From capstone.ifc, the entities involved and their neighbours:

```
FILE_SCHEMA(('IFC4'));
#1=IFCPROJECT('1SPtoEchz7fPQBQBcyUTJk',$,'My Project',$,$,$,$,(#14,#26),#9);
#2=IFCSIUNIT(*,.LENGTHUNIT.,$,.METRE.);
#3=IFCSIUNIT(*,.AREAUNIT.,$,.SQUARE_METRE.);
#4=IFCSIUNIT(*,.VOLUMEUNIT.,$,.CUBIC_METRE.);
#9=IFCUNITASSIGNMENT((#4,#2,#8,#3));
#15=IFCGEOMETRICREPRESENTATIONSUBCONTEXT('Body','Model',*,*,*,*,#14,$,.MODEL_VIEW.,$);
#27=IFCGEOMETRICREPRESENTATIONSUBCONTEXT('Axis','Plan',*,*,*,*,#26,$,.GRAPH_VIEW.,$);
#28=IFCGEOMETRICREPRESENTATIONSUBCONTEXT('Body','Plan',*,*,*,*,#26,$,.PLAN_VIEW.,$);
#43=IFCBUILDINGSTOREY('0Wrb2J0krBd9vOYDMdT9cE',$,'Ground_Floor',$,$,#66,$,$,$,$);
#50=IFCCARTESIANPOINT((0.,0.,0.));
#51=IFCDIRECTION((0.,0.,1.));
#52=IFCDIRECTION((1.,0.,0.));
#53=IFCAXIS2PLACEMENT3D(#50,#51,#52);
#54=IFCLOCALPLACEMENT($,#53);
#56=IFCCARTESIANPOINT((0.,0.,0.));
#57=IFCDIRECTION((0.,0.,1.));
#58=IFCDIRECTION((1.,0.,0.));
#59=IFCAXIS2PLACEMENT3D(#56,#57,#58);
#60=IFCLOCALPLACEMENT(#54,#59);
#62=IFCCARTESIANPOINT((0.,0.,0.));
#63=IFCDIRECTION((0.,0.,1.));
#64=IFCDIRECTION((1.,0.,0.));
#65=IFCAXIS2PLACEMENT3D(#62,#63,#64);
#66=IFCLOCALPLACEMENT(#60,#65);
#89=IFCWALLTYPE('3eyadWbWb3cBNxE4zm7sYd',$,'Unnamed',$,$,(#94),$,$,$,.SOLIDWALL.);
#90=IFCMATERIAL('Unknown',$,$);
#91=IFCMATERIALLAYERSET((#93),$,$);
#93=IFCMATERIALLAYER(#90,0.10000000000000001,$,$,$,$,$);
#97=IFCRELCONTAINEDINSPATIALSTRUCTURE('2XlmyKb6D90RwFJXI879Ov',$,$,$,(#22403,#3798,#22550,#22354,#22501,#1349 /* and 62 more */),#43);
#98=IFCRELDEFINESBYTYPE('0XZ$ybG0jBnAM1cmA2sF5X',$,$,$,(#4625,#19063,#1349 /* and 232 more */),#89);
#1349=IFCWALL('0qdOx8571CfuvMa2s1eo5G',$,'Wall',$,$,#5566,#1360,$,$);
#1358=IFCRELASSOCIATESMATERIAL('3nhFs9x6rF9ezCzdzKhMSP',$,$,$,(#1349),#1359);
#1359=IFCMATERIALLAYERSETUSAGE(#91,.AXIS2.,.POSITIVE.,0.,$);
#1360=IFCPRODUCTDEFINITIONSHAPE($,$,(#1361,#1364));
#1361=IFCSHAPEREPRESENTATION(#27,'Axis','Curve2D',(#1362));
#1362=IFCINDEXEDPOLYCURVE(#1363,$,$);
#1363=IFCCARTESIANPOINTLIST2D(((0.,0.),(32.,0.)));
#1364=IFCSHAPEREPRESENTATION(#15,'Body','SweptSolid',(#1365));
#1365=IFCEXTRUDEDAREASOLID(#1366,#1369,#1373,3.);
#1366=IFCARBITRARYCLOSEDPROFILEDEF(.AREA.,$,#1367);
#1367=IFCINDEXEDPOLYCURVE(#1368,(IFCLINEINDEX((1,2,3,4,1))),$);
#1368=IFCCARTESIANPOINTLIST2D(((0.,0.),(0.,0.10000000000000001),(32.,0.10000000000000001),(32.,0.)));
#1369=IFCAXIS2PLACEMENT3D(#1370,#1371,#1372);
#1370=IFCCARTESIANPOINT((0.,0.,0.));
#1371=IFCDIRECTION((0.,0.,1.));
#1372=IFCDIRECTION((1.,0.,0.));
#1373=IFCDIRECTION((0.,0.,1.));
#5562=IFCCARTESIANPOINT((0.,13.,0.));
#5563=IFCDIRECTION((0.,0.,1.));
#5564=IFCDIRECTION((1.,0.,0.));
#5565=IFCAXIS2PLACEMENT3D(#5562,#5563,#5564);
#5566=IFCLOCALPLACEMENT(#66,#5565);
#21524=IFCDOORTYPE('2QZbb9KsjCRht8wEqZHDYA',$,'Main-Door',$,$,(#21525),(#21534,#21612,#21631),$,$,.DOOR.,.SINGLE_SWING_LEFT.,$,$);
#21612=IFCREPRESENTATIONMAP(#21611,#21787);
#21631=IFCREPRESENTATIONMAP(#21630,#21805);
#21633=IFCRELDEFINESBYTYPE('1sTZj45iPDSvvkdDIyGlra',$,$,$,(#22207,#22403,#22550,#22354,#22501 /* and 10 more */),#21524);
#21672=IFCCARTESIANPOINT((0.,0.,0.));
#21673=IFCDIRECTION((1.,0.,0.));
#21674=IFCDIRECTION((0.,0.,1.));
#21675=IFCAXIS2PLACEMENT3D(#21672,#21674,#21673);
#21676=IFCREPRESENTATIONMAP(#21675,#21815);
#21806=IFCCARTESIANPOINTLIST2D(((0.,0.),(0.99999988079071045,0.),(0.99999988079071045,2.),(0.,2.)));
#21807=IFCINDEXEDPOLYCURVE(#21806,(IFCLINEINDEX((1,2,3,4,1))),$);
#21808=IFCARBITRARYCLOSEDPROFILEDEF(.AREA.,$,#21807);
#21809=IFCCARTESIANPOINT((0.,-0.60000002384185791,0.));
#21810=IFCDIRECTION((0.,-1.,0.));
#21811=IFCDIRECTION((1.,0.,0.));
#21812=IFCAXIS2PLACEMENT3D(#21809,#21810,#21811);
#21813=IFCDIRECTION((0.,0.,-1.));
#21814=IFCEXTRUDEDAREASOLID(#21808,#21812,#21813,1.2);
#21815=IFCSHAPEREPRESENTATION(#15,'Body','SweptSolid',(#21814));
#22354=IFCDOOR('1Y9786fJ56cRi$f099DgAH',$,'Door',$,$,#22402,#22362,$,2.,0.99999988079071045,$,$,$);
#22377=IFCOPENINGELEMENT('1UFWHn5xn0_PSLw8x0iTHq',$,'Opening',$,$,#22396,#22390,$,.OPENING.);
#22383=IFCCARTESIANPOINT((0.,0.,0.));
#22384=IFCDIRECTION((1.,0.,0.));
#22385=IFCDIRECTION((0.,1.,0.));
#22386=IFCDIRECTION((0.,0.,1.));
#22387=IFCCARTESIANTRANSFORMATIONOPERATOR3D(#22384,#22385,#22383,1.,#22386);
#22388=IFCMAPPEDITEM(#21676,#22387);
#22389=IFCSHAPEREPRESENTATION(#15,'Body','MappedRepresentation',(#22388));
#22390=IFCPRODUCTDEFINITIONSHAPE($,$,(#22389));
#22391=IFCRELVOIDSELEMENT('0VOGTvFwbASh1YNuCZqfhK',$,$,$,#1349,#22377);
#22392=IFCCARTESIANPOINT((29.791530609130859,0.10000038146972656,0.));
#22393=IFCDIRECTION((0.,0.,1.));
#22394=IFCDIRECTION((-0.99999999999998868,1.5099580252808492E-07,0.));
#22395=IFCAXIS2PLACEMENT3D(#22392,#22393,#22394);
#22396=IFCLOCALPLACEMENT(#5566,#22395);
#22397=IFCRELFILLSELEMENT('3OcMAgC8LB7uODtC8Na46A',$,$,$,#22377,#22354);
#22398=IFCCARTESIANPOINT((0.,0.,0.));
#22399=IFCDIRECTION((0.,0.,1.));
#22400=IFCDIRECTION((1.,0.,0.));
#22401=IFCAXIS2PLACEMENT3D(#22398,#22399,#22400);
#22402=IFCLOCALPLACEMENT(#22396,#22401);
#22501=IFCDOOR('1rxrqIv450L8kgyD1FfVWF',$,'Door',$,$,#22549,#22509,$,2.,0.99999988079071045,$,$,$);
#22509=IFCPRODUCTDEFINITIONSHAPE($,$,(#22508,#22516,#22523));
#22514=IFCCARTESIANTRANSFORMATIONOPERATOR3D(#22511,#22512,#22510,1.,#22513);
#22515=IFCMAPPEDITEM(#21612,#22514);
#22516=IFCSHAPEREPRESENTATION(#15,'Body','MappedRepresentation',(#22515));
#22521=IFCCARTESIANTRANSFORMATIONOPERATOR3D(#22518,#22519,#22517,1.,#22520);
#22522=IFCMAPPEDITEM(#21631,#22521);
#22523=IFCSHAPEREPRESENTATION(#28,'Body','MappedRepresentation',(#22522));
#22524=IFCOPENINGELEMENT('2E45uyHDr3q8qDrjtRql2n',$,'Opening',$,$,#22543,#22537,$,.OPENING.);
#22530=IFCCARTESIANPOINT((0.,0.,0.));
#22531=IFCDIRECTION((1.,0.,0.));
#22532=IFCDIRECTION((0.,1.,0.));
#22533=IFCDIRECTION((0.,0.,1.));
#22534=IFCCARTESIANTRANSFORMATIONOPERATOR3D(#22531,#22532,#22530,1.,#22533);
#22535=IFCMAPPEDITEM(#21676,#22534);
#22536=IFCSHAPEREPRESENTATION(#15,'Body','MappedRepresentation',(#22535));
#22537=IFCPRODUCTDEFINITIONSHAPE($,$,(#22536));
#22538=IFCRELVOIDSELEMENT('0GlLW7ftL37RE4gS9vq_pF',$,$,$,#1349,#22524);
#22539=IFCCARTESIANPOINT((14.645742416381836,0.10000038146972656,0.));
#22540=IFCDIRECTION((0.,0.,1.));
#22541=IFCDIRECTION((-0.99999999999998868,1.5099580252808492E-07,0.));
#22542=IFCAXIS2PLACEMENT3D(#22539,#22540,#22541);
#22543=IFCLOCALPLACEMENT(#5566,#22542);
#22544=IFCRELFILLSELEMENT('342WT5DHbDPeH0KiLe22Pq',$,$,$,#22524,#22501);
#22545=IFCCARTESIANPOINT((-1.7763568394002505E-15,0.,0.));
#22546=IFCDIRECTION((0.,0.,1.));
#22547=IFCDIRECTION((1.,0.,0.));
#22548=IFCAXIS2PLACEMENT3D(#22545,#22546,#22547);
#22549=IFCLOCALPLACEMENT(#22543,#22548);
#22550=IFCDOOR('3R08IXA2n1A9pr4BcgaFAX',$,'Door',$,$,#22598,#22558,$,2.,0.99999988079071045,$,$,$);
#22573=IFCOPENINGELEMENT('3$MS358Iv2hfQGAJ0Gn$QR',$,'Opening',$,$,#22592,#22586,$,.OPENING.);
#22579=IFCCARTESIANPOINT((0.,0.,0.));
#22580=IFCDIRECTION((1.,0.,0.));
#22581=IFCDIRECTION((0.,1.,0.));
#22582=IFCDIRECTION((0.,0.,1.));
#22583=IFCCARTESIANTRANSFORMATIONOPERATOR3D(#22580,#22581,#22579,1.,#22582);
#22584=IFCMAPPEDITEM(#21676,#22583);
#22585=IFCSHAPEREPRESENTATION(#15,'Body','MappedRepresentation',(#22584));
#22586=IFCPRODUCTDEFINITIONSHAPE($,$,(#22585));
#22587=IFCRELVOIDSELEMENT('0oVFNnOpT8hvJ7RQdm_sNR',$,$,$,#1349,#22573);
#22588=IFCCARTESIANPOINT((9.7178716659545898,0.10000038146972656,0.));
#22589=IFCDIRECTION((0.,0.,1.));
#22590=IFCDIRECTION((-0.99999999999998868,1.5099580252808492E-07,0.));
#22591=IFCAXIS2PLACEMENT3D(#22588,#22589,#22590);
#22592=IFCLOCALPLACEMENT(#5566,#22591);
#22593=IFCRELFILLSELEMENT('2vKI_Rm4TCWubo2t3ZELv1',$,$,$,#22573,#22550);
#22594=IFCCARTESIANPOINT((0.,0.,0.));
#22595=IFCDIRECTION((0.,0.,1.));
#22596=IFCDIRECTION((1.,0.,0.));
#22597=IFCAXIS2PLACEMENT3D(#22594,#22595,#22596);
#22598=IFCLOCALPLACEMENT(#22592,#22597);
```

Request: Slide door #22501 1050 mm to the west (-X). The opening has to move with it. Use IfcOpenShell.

```python
import ifcopenshell
import ifcopenshell.api.geometry
import ifcopenshell.util.placement

model = ifcopenshell.open("capstone.ifc")

door = model.by_id(22501)
opening = door.FillsVoids[0].RelatingOpeningElement
wall = opening.VoidsElements[0].RelatingBuildingElement

wall_matrix = ifcopenshell.util.placement.get_local_placement(wall.ObjectPlacement)
shift = wall_matrix[:3, 0] * -1.05
before = ifcopenshell.util.placement.get_local_placement(door.ObjectPlacement)[:3, 3].copy()

# The door is placed relative to its opening, so it follows when the opening moves.
matrix = ifcopenshell.util.placement.get_local_placement(opening.ObjectPlacement)
matrix[:3, 3] += shift
ifcopenshell.api.geometry.edit_object_placement(
    model, product=opening, matrix=matrix, is_si=False, should_transform_children=True
)

after = ifcopenshell.util.placement.get_local_placement(door.ObjectPlacement)[:3, 3]
print("door moved by", (after - before).round(3) + 0.0)

model.write("capstone_edited.ifc")
```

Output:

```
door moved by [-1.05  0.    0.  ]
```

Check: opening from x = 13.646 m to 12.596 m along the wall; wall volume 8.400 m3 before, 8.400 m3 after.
